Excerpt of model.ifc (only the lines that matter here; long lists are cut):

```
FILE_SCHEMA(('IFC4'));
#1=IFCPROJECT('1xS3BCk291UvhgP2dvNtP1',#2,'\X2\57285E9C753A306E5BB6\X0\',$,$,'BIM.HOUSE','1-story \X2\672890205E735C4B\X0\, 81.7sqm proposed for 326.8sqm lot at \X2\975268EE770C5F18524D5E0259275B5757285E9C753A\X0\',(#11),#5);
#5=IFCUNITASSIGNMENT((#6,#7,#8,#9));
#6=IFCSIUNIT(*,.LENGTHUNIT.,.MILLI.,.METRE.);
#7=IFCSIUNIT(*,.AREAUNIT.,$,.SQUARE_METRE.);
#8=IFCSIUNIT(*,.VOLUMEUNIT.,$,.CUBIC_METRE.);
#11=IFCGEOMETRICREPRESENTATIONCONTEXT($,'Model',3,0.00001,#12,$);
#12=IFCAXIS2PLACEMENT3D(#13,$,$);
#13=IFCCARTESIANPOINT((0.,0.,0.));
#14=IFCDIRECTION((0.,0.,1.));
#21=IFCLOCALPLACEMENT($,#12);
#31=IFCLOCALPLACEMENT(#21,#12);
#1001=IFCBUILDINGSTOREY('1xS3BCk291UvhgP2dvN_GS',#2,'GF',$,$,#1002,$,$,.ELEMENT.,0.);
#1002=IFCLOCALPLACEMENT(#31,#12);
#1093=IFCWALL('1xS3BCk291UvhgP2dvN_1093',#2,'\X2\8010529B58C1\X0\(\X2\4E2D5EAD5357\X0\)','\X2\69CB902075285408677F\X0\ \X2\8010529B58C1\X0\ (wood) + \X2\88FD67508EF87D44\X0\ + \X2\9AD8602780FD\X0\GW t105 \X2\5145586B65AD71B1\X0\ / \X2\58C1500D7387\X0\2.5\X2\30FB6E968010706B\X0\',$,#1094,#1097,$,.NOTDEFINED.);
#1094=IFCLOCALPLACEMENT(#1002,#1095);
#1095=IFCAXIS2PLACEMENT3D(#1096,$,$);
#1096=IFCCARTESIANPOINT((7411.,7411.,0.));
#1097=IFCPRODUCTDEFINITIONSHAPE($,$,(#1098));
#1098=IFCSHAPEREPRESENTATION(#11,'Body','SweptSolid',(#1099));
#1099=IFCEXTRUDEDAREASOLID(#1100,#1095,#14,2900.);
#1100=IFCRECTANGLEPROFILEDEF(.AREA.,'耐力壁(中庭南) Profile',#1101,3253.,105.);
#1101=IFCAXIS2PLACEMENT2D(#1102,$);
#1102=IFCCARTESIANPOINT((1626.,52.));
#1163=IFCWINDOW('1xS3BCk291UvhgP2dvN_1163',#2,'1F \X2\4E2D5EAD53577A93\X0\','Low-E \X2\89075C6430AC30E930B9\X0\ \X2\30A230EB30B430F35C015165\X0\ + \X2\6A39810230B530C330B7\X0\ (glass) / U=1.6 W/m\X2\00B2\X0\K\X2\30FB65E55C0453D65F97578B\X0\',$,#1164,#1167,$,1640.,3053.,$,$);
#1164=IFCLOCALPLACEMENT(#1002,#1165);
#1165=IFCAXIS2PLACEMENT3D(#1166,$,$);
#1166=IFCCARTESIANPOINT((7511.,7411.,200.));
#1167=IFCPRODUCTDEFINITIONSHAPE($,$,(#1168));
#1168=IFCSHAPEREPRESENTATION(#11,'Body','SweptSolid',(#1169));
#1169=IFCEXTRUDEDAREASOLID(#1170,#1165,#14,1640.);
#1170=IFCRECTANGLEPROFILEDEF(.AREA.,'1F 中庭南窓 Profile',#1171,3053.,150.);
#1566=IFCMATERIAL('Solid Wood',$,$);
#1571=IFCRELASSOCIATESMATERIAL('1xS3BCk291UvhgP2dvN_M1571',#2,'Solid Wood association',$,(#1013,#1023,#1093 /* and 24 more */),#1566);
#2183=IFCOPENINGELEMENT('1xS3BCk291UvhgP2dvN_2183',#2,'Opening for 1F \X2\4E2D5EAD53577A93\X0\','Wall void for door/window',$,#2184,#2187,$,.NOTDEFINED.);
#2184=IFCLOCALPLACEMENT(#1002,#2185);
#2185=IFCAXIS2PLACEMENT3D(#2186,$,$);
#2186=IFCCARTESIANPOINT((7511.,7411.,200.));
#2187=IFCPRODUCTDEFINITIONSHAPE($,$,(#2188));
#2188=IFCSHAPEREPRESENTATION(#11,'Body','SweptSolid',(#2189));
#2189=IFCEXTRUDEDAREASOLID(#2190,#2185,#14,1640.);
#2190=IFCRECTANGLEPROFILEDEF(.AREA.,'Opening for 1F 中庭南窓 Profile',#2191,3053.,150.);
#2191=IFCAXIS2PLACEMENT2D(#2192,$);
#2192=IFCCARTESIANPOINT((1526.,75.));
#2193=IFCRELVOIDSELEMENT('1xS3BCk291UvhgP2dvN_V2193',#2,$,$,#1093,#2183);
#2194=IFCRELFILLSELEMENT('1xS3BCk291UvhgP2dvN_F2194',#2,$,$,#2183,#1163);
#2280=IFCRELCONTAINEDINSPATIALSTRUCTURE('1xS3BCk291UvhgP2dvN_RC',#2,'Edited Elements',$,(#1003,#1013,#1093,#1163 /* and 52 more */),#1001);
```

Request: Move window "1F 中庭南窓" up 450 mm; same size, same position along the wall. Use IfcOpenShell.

```python
import numpy as np
import ifcopenshell
import ifcopenshell.api.geometry
import ifcopenshell.util.placement
import ifcopenshell.util.unit

model = ifcopenshell.open("model.ifc")
unit_scale = ifcopenshell.util.unit.calculate_unit_scale(model)

window = model.by_guid("1xS3BCk291UvhgP2dvN_1163")
opening = window.FillsVoids[0].RelatingOpeningElement
dz = 0.45 / unit_scale

shift = np.array([0.0, 0.0, dz])
# The window is not placed relative to its opening, so move both.
for product in (opening, window):
    matrix = ifcopenshell.util.placement.get_local_placement(product.ObjectPlacement)
    matrix[:3, 3] += shift
    ifcopenshell.api.geometry.edit_object_placement(model, product=product, matrix=matrix, is_si=False)

print(f"moved by {dz * unit_scale:+.3f} m")

model.write("model-out.ifc")
```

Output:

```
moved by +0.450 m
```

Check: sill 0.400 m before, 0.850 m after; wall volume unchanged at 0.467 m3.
